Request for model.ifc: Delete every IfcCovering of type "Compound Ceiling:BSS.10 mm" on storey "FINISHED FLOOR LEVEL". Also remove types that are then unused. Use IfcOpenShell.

First a look at what the model holds.

```python
import ifcopenshell
import ifcopenshell.util.element

model = ifcopenshell.open("model.ifc")
print(model.schema)
storey = next(s for s in model.by_type("IfcBuildingStorey") if s.Name == "FINISHED FLOOR LEVEL")
coverings = [e for e in ifcopenshell.util.element.get_decomposition(storey) if e.is_a("IfcCovering")]
seen = {}
for e in coverings:
    element_type = ifcopenshell.util.element.get_type(e)
    name = element_type.Name if element_type not in (None, e) else None
    seen[name] = seen.get(name, 0) + 1
for name, count in sorted(seen.items(), key=str):
    print(count, "x", name)
```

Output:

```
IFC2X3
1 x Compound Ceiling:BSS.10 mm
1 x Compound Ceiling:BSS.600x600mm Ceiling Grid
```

```python
import ifcopenshell
import ifcopenshell.api.root
import ifcopenshell.util.element

model = ifcopenshell.open("model.ifc")

storey = next(s for s in model.by_type("IfcBuildingStorey") if s.Name == "FINISHED FLOOR LEVEL")
coverings = [e for e in ifcopenshell.util.element.get_decomposition(storey) if e.is_a("IfcCovering")]
targets = [e for e in coverings if (t := ifcopenshell.util.element.get_type(e)) not in (None, e) and t.Name == "Compound Ceiling:BSS.10 mm"]
types = {ifcopenshell.util.element.get_type(e) for e in targets} - {None, *targets}

for e in targets:
    ifcopenshell.api.root.remove_product(model, product=e)
print(len(targets), "removed")

unused = [t for t in types if not ifcopenshell.util.element.get_types(t)]
for t in unused:
    ifcopenshell.api.root.remove_product(model, product=t)
print(len(unused), "unused types removed")

model.write("model-out.ifc")
```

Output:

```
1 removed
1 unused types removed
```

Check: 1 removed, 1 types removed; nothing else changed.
